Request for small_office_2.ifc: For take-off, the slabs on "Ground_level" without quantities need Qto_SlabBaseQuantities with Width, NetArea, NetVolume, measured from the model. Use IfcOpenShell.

First a look at what the model holds.

```python
import ifcopenshell
import ifcopenshell.util.element
import ifcopenshell.util.unit

model = ifcopenshell.open("small_office_2.ifc")
print(model.schema)
for unit_type in ("LENGTHUNIT", "AREAUNIT", "VOLUMEUNIT"):
    print(unit_type, ifcopenshell.util.unit.calculate_unit_scale(model, unit_type))
storey = next(s for s in model.by_type("IfcBuildingStorey") if s.Name == "Ground_level")
slabs = [e for e in ifcopenshell.util.element.get_decomposition(storey) if e.is_a("IfcSlab")]
for e in sorted(slabs, key=lambda e: e.id()):
    print(e.id(), e.is_a(), e.Name, list(ifcopenshell.util.element.get_psets(e, qtos_only=True)), sep=" | ")
```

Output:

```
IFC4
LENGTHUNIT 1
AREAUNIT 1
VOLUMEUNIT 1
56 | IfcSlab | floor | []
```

```python
import ifcopenshell
import ifcopenshell.api.pset
import ifcopenshell.geom
import ifcopenshell.util.element
import ifcopenshell.util.shape
import ifcopenshell.util.unit

model = ifcopenshell.open("small_office_2.ifc")
unit_scale = ifcopenshell.util.unit.calculate_unit_scale(model)
area_scale = ifcopenshell.util.unit.calculate_unit_scale(model, "AREAUNIT")
volume_scale = ifcopenshell.util.unit.calculate_unit_scale(model, "VOLUMEUNIT")
settings = ifcopenshell.geom.settings()

storey = next(s for s in model.by_type("IfcBuildingStorey") if s.Name == "Ground_level")
slabs = [e for e in ifcopenshell.util.element.get_decomposition(storey) if e.is_a("IfcSlab")]

for e in sorted(slabs, key=lambda e: e.id()):
    if ifcopenshell.util.element.get_psets(e, qtos_only=True, should_inherit=False):
        continue
    # Geometry comes back in metres, in the element's own axes.
    shape = ifcopenshell.geom.create_shape(settings, e)
    values = {
        "Width": ifcopenshell.util.shape.get_z(shape.geometry) / unit_scale,
        "NetArea": ifcopenshell.util.shape.get_footprint_area(shape.geometry) / area_scale,
        "NetVolume": ifcopenshell.util.shape.get_volume(shape.geometry) / volume_scale,
    }
    qto = ifcopenshell.api.pset.add_qto(model, product=e, name="Qto_SlabBaseQuantities")
    ifcopenshell.api.pset.edit_qto(model, qto=qto, properties=values)
    print(e.id(), {k: round(v, 3) for k, v in values.items()})

model.write("small_office_2-out.ifc")
```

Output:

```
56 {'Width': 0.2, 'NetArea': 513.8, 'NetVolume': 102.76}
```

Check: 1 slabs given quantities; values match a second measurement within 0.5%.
